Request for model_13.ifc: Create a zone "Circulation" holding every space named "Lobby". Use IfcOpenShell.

First a look at what the model holds.

```python
import ifcopenshell

model = ifcopenshell.open("model_13.ifc")
print(model.schema)
seen = {}
for space in model.by_type("IfcSpace"):
    seen[space.LongName] = seen.get(space.LongName, 0) + 1
for name, count in sorted(seen.items(), key=str):
    print(count, "x", name)
print("zones:", [z.Name for z in model.by_type("IfcZone")][:20])
```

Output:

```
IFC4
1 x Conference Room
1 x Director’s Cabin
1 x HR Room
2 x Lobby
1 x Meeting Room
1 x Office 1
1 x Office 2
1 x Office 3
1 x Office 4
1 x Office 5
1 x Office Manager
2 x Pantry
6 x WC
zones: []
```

```python
import ifcopenshell
import ifcopenshell.api.group
import ifcopenshell.api.root

model = ifcopenshell.open("model_13.ifc")

names = {"Lobby"}
spaces = [s for s in model.by_type("IfcSpace") if s.LongName in names]

zone = ifcopenshell.api.root.create_entity(model, ifc_class="IfcZone", name="Circulation")
ifcopenshell.api.group.assign_group(model, products=spaces, group=zone)
print(len(spaces), "spaces in", zone.Name)

model.write("model_13_edited.ifc")
```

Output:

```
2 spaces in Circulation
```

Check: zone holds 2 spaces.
